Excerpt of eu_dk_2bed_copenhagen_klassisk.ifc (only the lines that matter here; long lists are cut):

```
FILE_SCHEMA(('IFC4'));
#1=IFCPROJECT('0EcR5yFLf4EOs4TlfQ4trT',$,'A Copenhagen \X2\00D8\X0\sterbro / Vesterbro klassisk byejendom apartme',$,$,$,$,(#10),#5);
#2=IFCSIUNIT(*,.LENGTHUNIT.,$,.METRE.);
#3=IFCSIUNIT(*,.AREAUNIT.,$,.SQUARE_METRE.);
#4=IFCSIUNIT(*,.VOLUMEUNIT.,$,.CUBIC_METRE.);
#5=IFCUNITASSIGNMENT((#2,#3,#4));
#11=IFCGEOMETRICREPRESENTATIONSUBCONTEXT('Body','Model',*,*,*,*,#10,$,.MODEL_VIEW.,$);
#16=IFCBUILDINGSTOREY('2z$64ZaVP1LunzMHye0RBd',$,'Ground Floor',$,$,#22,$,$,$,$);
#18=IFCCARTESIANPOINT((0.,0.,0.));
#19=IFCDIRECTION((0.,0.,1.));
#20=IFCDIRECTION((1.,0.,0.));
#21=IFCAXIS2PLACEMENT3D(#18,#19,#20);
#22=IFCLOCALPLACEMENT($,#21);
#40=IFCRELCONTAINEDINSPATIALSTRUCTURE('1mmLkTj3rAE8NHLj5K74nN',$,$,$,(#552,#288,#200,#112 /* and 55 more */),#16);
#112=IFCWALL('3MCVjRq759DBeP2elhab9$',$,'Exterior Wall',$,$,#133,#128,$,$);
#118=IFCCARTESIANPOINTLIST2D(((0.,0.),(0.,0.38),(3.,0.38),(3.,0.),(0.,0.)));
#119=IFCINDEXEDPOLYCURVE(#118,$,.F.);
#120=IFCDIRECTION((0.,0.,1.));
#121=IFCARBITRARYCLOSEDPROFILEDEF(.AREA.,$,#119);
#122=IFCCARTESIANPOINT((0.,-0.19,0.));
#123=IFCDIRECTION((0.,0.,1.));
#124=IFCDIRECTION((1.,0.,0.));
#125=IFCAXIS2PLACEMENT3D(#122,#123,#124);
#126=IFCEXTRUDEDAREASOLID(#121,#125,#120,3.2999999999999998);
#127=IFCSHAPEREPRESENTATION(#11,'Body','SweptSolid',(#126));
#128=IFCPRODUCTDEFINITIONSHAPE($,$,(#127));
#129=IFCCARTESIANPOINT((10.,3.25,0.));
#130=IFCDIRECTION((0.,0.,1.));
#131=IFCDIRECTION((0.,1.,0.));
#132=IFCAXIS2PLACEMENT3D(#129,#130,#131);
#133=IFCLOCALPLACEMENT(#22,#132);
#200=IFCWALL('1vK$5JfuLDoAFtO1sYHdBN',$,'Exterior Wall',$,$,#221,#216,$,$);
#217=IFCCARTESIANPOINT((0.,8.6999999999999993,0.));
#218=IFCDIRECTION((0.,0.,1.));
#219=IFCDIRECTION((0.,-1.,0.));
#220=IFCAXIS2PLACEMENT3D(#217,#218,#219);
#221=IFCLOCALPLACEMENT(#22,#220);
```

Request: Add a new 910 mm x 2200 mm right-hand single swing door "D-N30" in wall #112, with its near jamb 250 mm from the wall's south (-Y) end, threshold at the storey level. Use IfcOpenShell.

```python
import numpy as np
import ifcopenshell
import ifcopenshell.api.feature
import ifcopenshell.api.geometry
import ifcopenshell.api.root
import ifcopenshell.api.spatial
import ifcopenshell.geom
import ifcopenshell.util.element
import ifcopenshell.util.placement
import ifcopenshell.util.representation
import ifcopenshell.util.shape
import ifcopenshell.util.unit

model = ifcopenshell.open("eu_dk_2bed_copenhagen_klassisk.ifc")
unit_scale = ifcopenshell.util.unit.calculate_unit_scale(model)
settings = ifcopenshell.geom.settings()


def volume(element):
    """Net volume in cubic metres, openings subtracted."""
    shape = ifcopenshell.geom.create_shape(settings, element)
    return ifcopenshell.util.shape.get_volume(shape.geometry)


wall = model.by_guid("3MCVjRq759DBeP2elhab9$")
storey = ifcopenshell.util.element.get_container(wall, ifc_class="IfcBuildingStorey")
context = ifcopenshell.util.representation.get_context(model, "Model", "Body", "MODEL_VIEW")
before = volume(wall)

width, height, from_end, sill = 0.91, 2.2, 0.25, 0.0  # metres

# The wall runs along its own X axis, and the end named is its -X end.
wall_shape = ifcopenshell.geom.create_shape(settings, wall)
x, y, z = ifcopenshell.util.shape.get_vertices(wall_shape.geometry).T
start = x.min() + from_end
face, thickness = float(y.min()), float(y.max() - y.min())
wall_matrix = ifcopenshell.util.placement.get_local_placement(wall.ObjectPlacement)
level = ifcopenshell.util.placement.get_local_placement(storey.ObjectPlacement)[2, 3]


def in_wall(x, y):
    """Placement at x, y metres in the wall's axes, at sill height."""
    matrix = wall_matrix.copy()
    matrix[:, 3] = wall_matrix @ np.array([x / unit_scale, y / unit_scale, 0.0, 1.0])
    matrix[2, 3] = level + sill / unit_scale
    return matrix


# Opening: a box that overshoots both wall faces by 50 mm.
opening = ifcopenshell.api.root.create_entity(model, ifc_class="IfcOpeningElement", predefined_type="OPENING")
box = ifcopenshell.api.geometry.add_wall_representation(
    model, context=context, length=width, height=height, thickness=thickness + 0.1
)
ifcopenshell.api.geometry.assign_representation(model, product=opening, representation=box)
ifcopenshell.api.geometry.edit_object_placement(model, product=opening, matrix=in_wall(start, face - 0.05), is_si=False)
ifcopenshell.api.feature.add_feature(model, feature=opening, element=wall)

door = ifcopenshell.api.root.create_entity(model, ifc_class="IfcDoor", name="D-N30", predefined_type="DOOR")
door.OverallWidth, door.OverallHeight = width / unit_scale, height / unit_scale
door.OperationType = "SINGLE_SWING_RIGHT"
body = ifcopenshell.api.geometry.add_door_representation(
    model,
    context=context,
    overall_width=door.OverallWidth,
    overall_height=door.OverallHeight,
    operation_type="SINGLE_SWING_RIGHT",
    lining_properties={"LiningDepth": thickness / unit_scale, "ThresholdDepth": thickness / unit_scale},
)
ifcopenshell.api.geometry.assign_representation(model, product=door, representation=body)
ifcopenshell.api.spatial.assign_container(model, products=[door], relating_structure=storey)
ifcopenshell.api.feature.add_filling(model, opening=opening, element=door)

# The lining spans the wall, so the door starts at the wall face.
ifcopenshell.api.geometry.edit_object_placement(model, product=door, matrix=in_wall(start, face), is_si=False)

after = volume(wall)

print(f"wall volume {before:.3f} -> {after:.3f} m3")

model.write("eu_dk_2bed_copenhagen_klassisk_rev.ifc")
```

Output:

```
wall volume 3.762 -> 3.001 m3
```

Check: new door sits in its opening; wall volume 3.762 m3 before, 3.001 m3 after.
